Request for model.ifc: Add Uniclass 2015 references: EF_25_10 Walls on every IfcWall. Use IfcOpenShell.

First a look at what the model holds.

```python
import ifcopenshell

model = ifcopenshell.open("model.ifc")
print(model.schema)
print("classifications:", [c.Name for c in model.by_type("IfcClassification")])
for ifc_class in ("IfcDoor", "IfcRoof", "IfcStair", "IfcWall", "IfcWindow"):
    print(ifc_class, len(model.by_type(ifc_class)))
```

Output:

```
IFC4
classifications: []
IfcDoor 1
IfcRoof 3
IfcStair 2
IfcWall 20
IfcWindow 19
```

```python
import ifcopenshell
import ifcopenshell.api.classification

model = ifcopenshell.open("model.ifc")

system = ifcopenshell.api.classification.add_classification(model, classification="Uniclass 2015")

codes = {
    "IfcWall": ("EF_25_10", "Walls"),
}
for ifc_class, (code, name) in codes.items():
    products = model.by_type(ifc_class)
    ifcopenshell.api.classification.add_reference(
        model, products=products, classification=system, identification=code, name=name
    )
    print(code, len(products))

model.write("model_v2.ifc")
```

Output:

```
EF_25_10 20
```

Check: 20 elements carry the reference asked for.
